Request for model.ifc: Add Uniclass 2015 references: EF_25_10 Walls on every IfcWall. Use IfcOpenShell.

First a look at what the model holds.

```python
import ifcopenshell

model = ifcopenshell.open("model.ifc")
print(model.schema)
print("classifications:", [c.Name for c in model.by_type("IfcClassification")])
for ifc_class in ("IfcDoor", "IfcRoof", "IfcStair", "IfcWall", "IfcWindow"):
    print(ifc_class, len(model.by_type(ifc_class)))
```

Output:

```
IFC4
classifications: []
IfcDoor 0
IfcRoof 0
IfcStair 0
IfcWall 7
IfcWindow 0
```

```python
import ifcopenshell
import ifcopenshell.api.classification

model = ifcopenshell.open("model.ifc")

system = ifcopenshell.api.classification.add_classification(model, classification="Uniclass 2015")

codes = {
    "IfcWall": ("EF_25_10", "Walls"),
}
for ifc_class, (code, name) in codes.items():
    products = model.by_type(ifc_class)
    ifcopenshell.api.classification.add_reference(
        model, products=products, classification=system, identification=code, name=name
    )
    print(code, len(products))

model.write("model-out.ifc")
```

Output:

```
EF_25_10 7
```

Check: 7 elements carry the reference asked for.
